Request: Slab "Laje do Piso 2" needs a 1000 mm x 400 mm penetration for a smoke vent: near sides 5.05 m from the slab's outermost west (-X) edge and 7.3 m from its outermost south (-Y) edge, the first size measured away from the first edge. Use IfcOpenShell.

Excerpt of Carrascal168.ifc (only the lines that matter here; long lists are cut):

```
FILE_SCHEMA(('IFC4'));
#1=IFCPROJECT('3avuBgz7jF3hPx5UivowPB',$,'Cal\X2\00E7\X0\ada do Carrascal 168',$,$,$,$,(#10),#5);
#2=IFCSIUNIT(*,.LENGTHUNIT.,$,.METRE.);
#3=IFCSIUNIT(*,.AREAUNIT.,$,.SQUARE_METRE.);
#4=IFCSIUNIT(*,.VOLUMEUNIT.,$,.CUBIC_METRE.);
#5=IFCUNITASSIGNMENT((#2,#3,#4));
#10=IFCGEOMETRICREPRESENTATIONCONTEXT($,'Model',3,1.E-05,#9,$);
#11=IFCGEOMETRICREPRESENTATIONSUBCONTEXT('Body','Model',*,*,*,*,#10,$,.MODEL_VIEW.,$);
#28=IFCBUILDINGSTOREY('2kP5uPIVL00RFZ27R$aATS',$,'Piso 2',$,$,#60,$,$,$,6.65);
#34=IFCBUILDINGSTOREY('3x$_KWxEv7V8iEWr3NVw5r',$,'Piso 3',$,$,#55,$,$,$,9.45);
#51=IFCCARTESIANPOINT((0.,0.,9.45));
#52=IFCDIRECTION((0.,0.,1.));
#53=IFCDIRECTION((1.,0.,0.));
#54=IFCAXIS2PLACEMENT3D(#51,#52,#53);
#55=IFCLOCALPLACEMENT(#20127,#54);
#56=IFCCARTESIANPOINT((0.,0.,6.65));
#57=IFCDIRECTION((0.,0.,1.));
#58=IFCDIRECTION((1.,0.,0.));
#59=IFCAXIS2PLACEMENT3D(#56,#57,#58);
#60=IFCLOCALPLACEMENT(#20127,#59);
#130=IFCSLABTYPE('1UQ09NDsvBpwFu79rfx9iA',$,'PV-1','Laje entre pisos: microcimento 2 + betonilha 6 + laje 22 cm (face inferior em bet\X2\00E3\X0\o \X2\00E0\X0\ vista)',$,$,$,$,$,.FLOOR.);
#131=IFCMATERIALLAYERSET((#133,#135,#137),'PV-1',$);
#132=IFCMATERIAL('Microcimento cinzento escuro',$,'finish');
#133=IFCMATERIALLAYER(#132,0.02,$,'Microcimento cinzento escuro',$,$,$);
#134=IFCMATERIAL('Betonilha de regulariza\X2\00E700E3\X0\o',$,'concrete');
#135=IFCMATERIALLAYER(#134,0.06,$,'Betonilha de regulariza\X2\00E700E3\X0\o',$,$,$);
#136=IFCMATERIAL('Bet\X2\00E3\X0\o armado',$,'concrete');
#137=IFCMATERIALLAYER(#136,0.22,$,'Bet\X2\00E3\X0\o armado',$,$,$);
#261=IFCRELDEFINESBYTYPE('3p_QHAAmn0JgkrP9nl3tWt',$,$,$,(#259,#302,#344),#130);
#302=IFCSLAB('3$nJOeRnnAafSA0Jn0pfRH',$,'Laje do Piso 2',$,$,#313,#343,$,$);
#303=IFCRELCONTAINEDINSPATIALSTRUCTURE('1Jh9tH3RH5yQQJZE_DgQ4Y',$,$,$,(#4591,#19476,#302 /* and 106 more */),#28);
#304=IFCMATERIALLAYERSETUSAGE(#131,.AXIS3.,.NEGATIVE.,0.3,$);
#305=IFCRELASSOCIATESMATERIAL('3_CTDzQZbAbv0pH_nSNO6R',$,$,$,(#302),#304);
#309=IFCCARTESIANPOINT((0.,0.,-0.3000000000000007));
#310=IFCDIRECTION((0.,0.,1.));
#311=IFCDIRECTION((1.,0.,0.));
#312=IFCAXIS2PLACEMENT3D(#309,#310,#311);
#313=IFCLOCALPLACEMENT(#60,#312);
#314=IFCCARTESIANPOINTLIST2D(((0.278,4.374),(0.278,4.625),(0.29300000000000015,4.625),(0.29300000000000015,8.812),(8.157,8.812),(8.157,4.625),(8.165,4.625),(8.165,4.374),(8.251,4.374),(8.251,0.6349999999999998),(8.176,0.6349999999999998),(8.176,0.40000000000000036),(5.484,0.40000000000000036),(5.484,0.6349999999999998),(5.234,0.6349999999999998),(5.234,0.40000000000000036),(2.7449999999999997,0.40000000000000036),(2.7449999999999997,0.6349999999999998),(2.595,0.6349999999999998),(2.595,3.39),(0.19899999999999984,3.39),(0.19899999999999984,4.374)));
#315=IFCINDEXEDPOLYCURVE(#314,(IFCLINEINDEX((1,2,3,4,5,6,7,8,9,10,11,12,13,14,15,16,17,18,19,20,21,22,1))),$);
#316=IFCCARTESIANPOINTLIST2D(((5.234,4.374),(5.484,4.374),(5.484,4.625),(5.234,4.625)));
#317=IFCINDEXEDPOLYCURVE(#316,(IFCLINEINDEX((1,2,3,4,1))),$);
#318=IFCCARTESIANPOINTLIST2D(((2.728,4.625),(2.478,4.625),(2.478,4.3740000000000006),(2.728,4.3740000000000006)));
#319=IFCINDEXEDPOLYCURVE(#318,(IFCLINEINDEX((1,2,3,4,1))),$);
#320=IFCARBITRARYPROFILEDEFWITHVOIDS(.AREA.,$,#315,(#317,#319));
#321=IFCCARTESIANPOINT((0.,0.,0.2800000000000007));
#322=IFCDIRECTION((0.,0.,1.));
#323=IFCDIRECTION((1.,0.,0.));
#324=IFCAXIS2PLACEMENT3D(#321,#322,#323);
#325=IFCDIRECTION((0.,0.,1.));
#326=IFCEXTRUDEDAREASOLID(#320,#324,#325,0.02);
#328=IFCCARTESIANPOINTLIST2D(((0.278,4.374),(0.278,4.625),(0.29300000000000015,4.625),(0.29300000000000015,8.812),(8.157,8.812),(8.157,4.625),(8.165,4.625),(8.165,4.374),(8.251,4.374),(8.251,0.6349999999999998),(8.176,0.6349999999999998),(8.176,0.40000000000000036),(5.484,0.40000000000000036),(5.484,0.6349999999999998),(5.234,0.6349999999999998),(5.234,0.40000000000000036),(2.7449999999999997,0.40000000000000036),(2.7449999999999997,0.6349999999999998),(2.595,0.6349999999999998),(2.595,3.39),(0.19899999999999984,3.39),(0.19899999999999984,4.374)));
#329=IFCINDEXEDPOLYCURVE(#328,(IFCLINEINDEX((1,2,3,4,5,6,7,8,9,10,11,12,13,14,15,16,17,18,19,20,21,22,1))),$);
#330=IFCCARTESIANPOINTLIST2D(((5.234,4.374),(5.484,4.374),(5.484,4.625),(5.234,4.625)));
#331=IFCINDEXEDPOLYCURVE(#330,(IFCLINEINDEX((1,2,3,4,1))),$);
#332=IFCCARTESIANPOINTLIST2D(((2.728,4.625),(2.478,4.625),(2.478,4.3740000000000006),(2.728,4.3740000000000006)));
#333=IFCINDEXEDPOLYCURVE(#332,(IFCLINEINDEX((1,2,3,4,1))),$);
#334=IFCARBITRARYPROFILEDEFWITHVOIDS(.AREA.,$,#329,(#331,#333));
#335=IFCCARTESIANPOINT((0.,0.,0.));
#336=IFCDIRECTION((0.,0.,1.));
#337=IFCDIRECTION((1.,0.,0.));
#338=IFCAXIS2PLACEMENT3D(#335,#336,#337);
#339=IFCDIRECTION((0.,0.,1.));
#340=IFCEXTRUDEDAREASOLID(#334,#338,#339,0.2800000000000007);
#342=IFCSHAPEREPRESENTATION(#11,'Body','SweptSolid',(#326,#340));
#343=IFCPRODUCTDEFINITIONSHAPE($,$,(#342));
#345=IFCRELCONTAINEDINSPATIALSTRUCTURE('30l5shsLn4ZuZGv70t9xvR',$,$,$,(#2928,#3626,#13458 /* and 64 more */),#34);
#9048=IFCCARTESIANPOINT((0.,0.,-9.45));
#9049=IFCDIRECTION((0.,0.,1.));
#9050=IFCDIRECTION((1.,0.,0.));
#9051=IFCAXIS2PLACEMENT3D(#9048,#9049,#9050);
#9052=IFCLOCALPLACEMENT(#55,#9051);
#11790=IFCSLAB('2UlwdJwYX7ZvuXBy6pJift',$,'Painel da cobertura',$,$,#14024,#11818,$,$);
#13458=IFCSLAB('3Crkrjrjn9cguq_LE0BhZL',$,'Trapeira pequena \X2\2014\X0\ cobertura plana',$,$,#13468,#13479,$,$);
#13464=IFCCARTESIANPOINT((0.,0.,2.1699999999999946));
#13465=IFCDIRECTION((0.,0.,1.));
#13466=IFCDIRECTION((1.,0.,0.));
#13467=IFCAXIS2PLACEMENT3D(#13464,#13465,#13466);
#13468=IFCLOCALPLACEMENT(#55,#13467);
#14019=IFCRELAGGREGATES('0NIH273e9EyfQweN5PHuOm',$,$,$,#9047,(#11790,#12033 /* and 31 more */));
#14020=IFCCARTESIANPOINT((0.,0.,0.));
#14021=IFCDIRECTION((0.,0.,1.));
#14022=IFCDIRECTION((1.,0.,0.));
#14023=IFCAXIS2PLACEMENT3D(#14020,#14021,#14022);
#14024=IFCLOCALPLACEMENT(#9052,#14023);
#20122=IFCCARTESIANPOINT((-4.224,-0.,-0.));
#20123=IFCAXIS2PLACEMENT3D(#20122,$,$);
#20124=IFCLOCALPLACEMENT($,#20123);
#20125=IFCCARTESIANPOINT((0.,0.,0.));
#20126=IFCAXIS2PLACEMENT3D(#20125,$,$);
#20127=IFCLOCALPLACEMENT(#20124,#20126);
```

```python
import numpy as np
import ifcopenshell
import ifcopenshell.api.feature
import ifcopenshell.api.geometry
import ifcopenshell.api.root
import ifcopenshell.geom
import ifcopenshell.util.placement
import ifcopenshell.util.representation
import ifcopenshell.util.shape
import ifcopenshell.util.unit

model = ifcopenshell.open("Carrascal168.ifc")
unit_scale = ifcopenshell.util.unit.calculate_unit_scale(model)
settings = ifcopenshell.geom.settings()


def volume(element):
    """Net volume in cubic metres, openings subtracted."""
    shape = ifcopenshell.geom.create_shape(settings, element)
    return ifcopenshell.util.shape.get_volume(shape.geometry)


slab = model.by_guid("3$nJOeRnnAafSA0Jn0pfRH")
before = volume(slab)

# Extent in the slab's own axes, in metres. The edges named are its -X and -Y sides.
slab_shape = ifcopenshell.geom.create_shape(settings, slab)
vertices = ifcopenshell.util.shape.get_vertices(slab_shape.geometry)
x_min, y_min, bottom = vertices.min(axis=0)
top = vertices[:, 2].max()

opening = ifcopenshell.api.root.create_entity(model, ifc_class="IfcOpeningElement", name="Smoke vent opening", predefined_type="OPENING")
context = ifcopenshell.util.representation.get_context(model, "Model", "Body", "MODEL_VIEW")
width, depth = 1, 0.4
outline = [(0.0, 0.0), (width, 0.0), (width, depth), (0.0, depth), (0.0, 0.0)]
# Overshoot both faces by 50 mm so the cut is clean.
shape = ifcopenshell.api.geometry.add_slab_representation(
    model, context=context, depth=top - bottom + 0.1, polyline=outline
)
ifcopenshell.api.geometry.assign_representation(model, product=opening, representation=shape)

matrix = ifcopenshell.util.placement.get_local_placement(slab.ObjectPlacement)
matrix[:, 3] = matrix @ np.append(np.array([x_min + 5.05, y_min + 7.3, bottom - 0.05]) / unit_scale, 1.0)
ifcopenshell.api.geometry.edit_object_placement(model, product=opening, matrix=matrix, is_si=False)
ifcopenshell.api.feature.add_feature(model, feature=opening, element=slab)

after = volume(slab)

print(f"slab volume {before:.3f} -> {after:.3f} m3")

model.write("Carrascal168_updated.ifc")
```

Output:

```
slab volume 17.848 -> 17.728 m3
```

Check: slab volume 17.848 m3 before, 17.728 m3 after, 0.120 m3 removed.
